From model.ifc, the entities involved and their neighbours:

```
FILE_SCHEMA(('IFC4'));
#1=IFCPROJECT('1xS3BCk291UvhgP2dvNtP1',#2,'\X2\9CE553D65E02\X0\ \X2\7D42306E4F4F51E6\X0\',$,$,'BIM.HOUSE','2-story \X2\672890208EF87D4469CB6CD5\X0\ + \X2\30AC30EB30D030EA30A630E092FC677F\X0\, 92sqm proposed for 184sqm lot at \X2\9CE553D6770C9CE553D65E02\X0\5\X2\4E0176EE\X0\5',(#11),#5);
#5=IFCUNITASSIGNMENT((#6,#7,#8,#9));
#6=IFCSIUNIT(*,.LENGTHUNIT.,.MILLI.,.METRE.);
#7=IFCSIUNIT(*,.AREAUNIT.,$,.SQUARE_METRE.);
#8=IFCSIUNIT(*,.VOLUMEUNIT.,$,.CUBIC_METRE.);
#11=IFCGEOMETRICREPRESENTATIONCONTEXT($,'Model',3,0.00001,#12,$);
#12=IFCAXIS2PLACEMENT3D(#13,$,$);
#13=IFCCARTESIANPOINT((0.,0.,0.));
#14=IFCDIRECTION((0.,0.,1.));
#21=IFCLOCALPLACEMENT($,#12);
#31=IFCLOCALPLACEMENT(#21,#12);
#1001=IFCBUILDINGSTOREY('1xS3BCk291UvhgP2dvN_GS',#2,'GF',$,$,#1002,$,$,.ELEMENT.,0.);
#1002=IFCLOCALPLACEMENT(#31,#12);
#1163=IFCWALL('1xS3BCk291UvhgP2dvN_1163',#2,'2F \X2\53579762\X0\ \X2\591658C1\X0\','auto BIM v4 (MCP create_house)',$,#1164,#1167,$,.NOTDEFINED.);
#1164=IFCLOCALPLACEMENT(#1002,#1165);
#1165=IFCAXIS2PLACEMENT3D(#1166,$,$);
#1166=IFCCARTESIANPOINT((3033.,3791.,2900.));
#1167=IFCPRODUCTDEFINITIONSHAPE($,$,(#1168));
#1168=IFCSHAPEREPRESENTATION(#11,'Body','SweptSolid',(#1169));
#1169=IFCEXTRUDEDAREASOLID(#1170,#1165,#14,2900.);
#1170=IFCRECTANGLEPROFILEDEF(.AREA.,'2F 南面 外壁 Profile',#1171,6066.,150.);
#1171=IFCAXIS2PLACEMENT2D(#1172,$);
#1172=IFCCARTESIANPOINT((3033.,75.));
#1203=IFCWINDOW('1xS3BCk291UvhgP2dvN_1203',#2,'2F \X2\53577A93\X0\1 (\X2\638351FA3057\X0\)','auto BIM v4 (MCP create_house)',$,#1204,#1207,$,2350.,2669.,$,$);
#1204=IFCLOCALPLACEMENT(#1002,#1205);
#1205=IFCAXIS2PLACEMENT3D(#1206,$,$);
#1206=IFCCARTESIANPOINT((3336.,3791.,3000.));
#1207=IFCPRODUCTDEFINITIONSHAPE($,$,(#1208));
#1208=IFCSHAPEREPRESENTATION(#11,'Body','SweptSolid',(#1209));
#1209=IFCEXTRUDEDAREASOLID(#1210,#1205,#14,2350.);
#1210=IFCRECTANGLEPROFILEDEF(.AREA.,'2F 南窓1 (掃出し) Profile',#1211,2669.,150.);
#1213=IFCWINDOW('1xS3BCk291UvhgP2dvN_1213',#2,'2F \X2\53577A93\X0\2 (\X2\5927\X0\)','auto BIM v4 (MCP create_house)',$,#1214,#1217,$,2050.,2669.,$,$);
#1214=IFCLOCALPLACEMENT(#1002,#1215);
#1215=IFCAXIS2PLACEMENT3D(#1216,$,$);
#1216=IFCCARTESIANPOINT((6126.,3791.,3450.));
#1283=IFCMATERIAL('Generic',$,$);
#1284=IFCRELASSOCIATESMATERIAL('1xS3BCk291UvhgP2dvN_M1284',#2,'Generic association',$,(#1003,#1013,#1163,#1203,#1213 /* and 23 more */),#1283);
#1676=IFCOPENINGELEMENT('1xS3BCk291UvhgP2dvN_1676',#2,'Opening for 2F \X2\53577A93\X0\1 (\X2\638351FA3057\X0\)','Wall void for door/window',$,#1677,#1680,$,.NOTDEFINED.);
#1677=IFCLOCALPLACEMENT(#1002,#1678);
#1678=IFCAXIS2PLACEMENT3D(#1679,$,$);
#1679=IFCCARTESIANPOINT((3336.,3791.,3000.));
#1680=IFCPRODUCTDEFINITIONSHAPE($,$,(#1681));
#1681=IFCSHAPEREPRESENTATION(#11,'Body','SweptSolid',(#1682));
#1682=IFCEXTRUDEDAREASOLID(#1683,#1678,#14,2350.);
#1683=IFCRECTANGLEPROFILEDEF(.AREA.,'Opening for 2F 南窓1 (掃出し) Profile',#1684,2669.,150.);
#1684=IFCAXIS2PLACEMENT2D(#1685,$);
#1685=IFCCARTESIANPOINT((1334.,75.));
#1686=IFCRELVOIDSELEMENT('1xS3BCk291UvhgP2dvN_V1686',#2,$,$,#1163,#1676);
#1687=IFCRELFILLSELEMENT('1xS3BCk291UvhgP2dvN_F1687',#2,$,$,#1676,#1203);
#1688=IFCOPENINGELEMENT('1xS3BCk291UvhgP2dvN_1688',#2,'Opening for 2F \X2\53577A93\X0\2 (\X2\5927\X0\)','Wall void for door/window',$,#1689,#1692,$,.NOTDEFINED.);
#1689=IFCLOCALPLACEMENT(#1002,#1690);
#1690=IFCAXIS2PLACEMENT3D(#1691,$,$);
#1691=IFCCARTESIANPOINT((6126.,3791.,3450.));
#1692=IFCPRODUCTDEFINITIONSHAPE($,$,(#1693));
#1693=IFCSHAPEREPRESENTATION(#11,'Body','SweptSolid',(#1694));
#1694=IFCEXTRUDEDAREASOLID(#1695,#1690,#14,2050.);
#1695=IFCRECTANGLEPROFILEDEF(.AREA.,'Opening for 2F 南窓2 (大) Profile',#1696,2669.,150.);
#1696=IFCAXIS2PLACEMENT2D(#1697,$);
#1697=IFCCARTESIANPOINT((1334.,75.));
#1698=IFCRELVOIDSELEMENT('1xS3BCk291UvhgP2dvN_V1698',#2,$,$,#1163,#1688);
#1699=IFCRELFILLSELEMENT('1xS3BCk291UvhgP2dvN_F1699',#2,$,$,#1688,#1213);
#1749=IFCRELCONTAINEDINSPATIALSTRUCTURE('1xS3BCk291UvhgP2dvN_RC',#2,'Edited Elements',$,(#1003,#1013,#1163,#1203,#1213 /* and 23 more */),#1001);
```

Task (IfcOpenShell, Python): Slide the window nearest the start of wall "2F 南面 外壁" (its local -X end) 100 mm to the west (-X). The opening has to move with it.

```python
import ifcopenshell
import ifcopenshell.api.geometry
import ifcopenshell.util.placement
import ifcopenshell.util.unit

model = ifcopenshell.open("model.ifc")
unit_scale = ifcopenshell.util.unit.calculate_unit_scale(model)

window = model.by_guid("1xS3BCk291UvhgP2dvN_1203")
opening = window.FillsVoids[0].RelatingOpeningElement
wall = opening.VoidsElements[0].RelatingBuildingElement

wall_matrix = ifcopenshell.util.placement.get_local_placement(wall.ObjectPlacement)
shift = wall_matrix[:3, 0] * -0.1 / unit_scale
before = ifcopenshell.util.placement.get_local_placement(window.ObjectPlacement)[:3, 3].copy()

# The window is not placed relative to its opening, so move both.
for product in (opening, window):
    matrix = ifcopenshell.util.placement.get_local_placement(product.ObjectPlacement)
    matrix[:3, 3] += shift
    ifcopenshell.api.geometry.edit_object_placement(model, product=product, matrix=matrix, is_si=False)

after = ifcopenshell.util.placement.get_local_placement(window.ObjectPlacement)[:3, 3]
print("window moved by", (after - before).round(3) + 0.0)

model.write("model_edited.ifc")
```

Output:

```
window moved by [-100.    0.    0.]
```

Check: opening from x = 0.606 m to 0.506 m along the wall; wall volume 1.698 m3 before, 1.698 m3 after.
